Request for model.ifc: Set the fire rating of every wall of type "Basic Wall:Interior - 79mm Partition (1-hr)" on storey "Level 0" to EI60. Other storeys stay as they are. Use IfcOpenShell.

First a look at what the model holds.

```python
import ifcopenshell
import ifcopenshell.util.element

model = ifcopenshell.open("model.ifc")
print(model.schema)
storey = next(s for s in model.by_type("IfcBuildingStorey") if s.Name == "Level 0")
walls = [e for e in ifcopenshell.util.element.get_decomposition(storey) if e.is_a("IfcWall")]
seen = {}
for e in walls:
    element_type = ifcopenshell.util.element.get_type(e)
    key = (element_type.Name if element_type != e and element_type else None, ifcopenshell.util.element.get_pset(e, "Pset_WallCommon", "FireRating"))
    seen[key] = seen.get(key, 0) + 1
for (name, value), count in sorted(seen.items(), key=str):
    print(count, "x", name, "|", value)
```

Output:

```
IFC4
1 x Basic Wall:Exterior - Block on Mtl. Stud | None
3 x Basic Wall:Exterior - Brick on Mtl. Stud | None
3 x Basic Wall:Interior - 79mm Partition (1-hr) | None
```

```python
import ifcopenshell
import ifcopenshell.api.pset
import ifcopenshell.util.element

model = ifcopenshell.open("model.ifc")

storey = next(s for s in model.by_type("IfcBuildingStorey") if s.Name == "Level 0")
walls = [e for e in ifcopenshell.util.element.get_decomposition(storey) if e.is_a("IfcWall")]

count = 0
for e in walls:
    element_type = ifcopenshell.util.element.get_type(e)
    if element_type in (None, e) or element_type.Name != "Basic Wall:Interior - 79mm Partition (1-hr)":
        continue
    # add_pset returns the element's existing set when there is one.
    pset = ifcopenshell.api.pset.add_pset(model, product=e, name="Pset_WallCommon")
    ifcopenshell.api.pset.edit_pset(model, pset=pset, properties={"FireRating": "EI60"})
    count += 1

print(count, "walls updated")

model.write("model_edited.ifc")
```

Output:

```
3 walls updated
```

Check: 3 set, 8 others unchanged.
